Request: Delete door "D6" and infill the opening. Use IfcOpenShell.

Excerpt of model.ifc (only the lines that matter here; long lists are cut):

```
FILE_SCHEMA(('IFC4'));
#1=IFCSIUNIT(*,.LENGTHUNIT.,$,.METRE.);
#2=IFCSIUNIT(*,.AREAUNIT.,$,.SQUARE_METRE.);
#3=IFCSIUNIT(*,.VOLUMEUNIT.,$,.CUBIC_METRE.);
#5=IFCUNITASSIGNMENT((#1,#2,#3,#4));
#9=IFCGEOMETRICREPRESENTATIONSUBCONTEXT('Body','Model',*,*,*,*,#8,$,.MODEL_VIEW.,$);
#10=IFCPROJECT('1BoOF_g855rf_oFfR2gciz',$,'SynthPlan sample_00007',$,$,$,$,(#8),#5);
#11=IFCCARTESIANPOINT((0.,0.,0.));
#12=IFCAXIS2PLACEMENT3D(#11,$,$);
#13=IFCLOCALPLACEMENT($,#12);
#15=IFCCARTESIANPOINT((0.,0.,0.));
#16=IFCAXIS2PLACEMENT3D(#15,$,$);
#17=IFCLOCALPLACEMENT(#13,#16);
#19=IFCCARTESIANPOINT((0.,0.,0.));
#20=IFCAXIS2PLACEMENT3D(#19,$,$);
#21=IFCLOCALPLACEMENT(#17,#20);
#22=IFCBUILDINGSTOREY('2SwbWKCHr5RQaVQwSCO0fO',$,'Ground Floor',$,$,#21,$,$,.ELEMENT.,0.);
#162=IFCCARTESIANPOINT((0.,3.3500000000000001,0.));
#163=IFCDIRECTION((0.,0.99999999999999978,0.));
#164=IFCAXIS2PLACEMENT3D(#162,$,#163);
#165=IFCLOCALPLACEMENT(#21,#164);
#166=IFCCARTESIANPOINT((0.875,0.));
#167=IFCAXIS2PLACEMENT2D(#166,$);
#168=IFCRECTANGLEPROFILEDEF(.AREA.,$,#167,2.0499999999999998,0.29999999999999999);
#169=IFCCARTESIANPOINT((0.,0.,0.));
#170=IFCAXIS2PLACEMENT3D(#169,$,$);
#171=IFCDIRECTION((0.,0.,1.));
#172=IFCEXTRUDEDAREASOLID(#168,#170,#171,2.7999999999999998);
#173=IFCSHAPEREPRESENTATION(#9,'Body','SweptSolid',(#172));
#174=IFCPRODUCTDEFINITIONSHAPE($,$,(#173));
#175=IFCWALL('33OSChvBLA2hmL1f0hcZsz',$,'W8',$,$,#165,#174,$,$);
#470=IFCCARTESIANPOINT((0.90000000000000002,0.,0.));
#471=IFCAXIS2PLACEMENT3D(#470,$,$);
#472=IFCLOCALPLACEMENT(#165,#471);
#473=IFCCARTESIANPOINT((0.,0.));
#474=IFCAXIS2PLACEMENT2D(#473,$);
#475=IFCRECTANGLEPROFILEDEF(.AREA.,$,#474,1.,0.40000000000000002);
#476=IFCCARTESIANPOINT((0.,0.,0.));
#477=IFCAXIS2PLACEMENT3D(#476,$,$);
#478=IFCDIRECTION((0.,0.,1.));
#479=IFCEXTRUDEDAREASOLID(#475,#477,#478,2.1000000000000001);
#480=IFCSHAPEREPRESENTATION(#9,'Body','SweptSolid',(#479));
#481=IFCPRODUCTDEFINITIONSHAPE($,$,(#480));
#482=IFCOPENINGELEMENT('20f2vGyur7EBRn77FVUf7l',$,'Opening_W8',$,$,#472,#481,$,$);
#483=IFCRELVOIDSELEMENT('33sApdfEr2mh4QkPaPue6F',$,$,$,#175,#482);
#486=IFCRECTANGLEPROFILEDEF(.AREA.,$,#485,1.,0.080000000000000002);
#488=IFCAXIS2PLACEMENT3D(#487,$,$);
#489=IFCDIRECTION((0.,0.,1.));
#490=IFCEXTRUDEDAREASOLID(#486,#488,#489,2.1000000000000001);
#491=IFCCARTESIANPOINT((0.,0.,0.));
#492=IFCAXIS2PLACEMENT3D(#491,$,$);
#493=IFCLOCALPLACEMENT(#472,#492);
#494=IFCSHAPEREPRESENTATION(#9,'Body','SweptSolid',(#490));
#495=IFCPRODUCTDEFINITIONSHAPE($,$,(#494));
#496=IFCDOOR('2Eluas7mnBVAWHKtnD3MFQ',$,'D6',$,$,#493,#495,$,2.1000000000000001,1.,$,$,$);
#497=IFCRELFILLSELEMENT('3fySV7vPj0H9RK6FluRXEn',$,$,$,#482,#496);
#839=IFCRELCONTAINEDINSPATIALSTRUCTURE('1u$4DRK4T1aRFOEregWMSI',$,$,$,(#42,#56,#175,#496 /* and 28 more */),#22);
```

```python
import ifcopenshell
import ifcopenshell.api.feature
import ifcopenshell.api.root
import ifcopenshell.geom
import ifcopenshell.util.shape

model = ifcopenshell.open("model.ifc")
settings = ifcopenshell.geom.settings()


def volume(element):
    """Net volume in cubic metres, openings subtracted."""
    shape = ifcopenshell.geom.create_shape(settings, element)
    return ifcopenshell.util.shape.get_volume(shape.geometry)


door = model.by_guid("2Eluas7mnBVAWHKtnD3MFQ")
opening = door.FillsVoids[0].RelatingOpeningElement
wall = opening.VoidsElements[0].RelatingBuildingElement
before = volume(wall)

ifcopenshell.api.root.remove_product(model, product=door)
ifcopenshell.api.feature.remove_feature(model, feature=opening)

after = volume(wall)

print(f"wall volume {before:.3f} -> {after:.3f} m3")

model.write("model-out.ifc")
```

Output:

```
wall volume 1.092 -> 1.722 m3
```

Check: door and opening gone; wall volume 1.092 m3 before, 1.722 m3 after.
